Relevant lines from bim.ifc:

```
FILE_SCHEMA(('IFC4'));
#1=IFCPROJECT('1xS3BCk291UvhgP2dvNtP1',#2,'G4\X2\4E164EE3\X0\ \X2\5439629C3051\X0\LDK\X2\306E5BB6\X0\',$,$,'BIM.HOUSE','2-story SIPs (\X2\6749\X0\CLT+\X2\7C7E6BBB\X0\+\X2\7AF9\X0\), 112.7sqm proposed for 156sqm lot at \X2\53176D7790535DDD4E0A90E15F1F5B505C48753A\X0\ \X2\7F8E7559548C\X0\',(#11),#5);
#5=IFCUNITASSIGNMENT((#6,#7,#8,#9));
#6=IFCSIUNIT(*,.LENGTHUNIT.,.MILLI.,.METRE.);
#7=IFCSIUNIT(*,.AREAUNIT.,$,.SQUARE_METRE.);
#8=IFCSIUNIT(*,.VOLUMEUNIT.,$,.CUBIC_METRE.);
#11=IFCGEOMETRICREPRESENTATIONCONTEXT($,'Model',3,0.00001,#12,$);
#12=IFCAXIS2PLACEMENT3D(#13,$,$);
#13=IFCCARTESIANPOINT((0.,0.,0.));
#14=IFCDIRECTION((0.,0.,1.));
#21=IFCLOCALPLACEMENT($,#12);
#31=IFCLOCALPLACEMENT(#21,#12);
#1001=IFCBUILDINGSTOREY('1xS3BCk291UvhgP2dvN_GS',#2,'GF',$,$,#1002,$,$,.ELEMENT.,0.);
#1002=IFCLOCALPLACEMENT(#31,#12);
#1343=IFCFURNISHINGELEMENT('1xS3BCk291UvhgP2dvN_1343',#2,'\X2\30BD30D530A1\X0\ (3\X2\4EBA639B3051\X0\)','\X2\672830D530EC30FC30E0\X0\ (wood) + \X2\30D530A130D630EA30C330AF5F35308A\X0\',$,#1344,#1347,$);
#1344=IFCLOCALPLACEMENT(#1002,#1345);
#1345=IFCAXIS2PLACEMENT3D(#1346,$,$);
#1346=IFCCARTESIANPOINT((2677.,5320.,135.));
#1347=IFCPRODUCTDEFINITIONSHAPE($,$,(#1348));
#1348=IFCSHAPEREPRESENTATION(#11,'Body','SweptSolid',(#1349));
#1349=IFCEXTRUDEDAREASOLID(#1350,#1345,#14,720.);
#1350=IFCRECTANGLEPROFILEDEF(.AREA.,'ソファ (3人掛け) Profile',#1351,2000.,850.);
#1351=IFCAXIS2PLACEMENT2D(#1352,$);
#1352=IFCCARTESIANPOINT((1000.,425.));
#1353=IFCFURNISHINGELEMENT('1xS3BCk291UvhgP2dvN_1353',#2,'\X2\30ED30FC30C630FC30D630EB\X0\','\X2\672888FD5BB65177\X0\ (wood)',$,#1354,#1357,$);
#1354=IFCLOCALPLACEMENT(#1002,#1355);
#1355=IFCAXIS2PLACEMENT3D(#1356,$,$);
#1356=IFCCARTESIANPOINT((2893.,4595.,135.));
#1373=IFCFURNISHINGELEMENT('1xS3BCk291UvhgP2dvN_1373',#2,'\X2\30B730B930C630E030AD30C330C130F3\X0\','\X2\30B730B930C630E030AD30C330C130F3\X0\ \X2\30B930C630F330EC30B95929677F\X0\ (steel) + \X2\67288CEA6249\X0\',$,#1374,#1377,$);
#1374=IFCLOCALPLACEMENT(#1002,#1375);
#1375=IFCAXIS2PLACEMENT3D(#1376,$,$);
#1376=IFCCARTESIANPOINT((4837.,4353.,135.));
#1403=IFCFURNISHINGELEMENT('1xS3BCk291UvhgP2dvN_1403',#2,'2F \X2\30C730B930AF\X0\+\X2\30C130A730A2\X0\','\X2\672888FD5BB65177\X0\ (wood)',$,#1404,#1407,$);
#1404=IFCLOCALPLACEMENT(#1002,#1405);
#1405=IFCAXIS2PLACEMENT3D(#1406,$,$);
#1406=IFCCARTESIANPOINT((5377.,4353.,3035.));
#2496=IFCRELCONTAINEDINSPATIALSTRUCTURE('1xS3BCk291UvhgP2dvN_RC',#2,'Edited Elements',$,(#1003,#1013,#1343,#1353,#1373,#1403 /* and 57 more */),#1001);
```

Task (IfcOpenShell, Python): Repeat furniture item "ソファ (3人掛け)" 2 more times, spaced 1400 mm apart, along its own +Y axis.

```python
import ifcopenshell
import ifcopenshell.api.geometry
import ifcopenshell.api.root
import ifcopenshell.util.element
import ifcopenshell.util.placement

model = ifcopenshell.open("bim.ifc")


def reuse_history(source, copy):
    """copy_class also copies each property set's owner history, people and application; keep the originals."""
    for rel in copy.IsDefinedBy:
        if rel.is_a("IfcRelDefinesByProperties") and (history := rel.RelatingPropertyDefinition.OwnerHistory):
            rel.RelatingPropertyDefinition.OwnerHistory = source.OwnerHistory
            ifcopenshell.util.element.remove_deep2(model, history)


source = model.by_id(1343)
base = ifcopenshell.util.placement.get_local_placement(source.ObjectPlacement)
step = base[:3, 1] * 1400.0

for i in range(1, 3):
    copy = ifcopenshell.api.root.copy_class(model, product=source)
    copy.Representation = ifcopenshell.util.element.copy_deep(
        model, source.Representation, exclude=["IfcGeometricRepresentationContext", "IfcRepresentationMap"]
    )
    reuse_history(source, copy)
    matrix = base.copy()
    matrix[:3, 3] += i * step
    print("added at", matrix[:3, 3].round(3) + 0.0)
    ifcopenshell.api.geometry.edit_object_placement(model, product=copy, matrix=matrix, is_si=False)

model.write("bim_v2.ifc")
```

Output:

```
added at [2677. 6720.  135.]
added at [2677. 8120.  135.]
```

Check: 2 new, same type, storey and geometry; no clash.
